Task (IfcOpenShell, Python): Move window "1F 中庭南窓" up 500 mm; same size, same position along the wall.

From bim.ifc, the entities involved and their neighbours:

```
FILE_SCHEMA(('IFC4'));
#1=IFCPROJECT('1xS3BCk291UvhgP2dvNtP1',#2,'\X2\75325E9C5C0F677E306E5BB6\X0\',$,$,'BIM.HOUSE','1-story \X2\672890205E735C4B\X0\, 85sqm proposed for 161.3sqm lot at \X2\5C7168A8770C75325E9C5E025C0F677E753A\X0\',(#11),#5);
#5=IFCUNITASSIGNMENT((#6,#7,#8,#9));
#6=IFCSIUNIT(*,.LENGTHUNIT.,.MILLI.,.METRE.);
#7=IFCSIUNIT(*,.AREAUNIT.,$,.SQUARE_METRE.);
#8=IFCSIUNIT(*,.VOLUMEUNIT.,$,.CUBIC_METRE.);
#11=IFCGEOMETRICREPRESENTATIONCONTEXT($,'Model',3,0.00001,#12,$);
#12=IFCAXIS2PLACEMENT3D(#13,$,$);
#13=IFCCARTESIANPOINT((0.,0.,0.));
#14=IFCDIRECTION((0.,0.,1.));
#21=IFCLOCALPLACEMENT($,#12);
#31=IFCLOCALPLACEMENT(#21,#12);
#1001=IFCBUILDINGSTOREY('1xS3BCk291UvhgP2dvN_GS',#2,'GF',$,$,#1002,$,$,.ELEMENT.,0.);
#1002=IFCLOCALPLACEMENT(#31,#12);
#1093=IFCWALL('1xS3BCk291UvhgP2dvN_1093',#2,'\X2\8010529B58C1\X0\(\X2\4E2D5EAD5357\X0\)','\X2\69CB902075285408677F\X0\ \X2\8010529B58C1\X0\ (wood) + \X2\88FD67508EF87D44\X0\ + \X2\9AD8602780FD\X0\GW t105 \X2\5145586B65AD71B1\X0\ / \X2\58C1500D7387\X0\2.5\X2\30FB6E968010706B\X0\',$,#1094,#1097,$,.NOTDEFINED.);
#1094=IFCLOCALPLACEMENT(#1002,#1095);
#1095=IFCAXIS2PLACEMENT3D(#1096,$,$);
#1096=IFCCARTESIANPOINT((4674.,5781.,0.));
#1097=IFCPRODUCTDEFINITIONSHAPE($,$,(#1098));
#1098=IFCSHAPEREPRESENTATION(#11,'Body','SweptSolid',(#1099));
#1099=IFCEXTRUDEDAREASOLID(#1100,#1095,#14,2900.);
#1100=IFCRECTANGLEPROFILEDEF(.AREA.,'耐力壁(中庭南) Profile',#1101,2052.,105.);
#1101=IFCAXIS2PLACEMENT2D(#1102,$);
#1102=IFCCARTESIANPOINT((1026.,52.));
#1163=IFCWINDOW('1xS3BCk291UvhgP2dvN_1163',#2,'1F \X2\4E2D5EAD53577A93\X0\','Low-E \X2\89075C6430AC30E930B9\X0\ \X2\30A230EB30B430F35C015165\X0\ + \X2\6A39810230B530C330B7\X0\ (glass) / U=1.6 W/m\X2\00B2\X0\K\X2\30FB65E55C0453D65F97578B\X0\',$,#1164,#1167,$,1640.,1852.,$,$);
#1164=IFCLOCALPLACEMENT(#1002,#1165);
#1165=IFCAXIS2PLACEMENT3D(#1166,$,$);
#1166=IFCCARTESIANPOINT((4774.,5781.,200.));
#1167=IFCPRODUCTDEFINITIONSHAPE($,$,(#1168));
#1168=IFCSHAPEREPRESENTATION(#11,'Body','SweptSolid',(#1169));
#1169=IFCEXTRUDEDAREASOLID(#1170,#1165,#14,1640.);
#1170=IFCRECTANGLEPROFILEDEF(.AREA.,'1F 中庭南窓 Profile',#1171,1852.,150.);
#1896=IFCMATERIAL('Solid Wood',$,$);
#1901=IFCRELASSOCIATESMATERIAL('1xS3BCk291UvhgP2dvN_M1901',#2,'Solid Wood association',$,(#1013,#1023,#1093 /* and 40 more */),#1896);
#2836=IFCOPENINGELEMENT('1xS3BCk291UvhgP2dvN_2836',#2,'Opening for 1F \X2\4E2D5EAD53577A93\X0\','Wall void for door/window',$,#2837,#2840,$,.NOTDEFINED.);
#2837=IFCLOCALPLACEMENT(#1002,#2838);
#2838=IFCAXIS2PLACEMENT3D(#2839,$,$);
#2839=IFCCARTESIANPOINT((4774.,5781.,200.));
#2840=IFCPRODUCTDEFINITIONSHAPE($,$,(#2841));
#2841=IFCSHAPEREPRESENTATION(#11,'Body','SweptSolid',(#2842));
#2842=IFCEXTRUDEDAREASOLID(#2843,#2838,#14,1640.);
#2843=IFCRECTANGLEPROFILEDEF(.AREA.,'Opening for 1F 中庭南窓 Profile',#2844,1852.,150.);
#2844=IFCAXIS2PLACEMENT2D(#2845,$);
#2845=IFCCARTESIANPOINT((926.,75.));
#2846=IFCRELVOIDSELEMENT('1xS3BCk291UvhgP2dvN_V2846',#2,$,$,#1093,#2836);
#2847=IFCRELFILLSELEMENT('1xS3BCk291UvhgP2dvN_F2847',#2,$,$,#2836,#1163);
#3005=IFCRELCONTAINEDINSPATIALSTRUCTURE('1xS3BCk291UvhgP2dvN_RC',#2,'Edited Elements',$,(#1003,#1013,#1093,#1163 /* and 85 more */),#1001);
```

```python
import numpy as np
import ifcopenshell
import ifcopenshell.api.geometry
import ifcopenshell.util.placement
import ifcopenshell.util.unit

model = ifcopenshell.open("bim.ifc")
unit_scale = ifcopenshell.util.unit.calculate_unit_scale(model)

window = model.by_guid("1xS3BCk291UvhgP2dvN_1163")
opening = window.FillsVoids[0].RelatingOpeningElement
dz = 0.5 / unit_scale

shift = np.array([0.0, 0.0, dz])
# The window is not placed relative to its opening, so move both.
for product in (opening, window):
    matrix = ifcopenshell.util.placement.get_local_placement(product.ObjectPlacement)
    matrix[:3, 3] += shift
    ifcopenshell.api.geometry.edit_object_placement(model, product=product, matrix=matrix, is_si=False)

print(f"moved by {dz * unit_scale:+.3f} m")

model.write("bim_edited.ifc")
```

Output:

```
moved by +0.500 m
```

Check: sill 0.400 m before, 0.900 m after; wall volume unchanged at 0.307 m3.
